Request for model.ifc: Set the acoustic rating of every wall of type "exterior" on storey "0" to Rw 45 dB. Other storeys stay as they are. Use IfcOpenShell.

First a look at what the model holds.

```python
import ifcopenshell
import ifcopenshell.util.element

model = ifcopenshell.open("model.ifc")
print(model.schema)
storey = next(s for s in model.by_type("IfcBuildingStorey") if s.Name == "0")
walls = [e for e in ifcopenshell.util.element.get_decomposition(storey) if e.is_a("IfcWall")]
seen = {}
for e in walls:
    element_type = ifcopenshell.util.element.get_type(e)
    key = (element_type.Name if element_type != e and element_type else None, ifcopenshell.util.element.get_pset(e, "Pset_WallCommon", "AcousticRating"))
    seen[key] = seen.get(key, 0) + 1
for (name, value), count in sorted(seen.items(), key=str):
    print(count, "x", name, "|", value)
```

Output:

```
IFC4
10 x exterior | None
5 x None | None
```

```python
import ifcopenshell
import ifcopenshell.api.pset
import ifcopenshell.util.element

model = ifcopenshell.open("model.ifc")

storey = next(s for s in model.by_type("IfcBuildingStorey") if s.Name == "0")
walls = [e for e in ifcopenshell.util.element.get_decomposition(storey) if e.is_a("IfcWall")]

count = 0
for e in walls:
    element_type = ifcopenshell.util.element.get_type(e)
    if element_type in (None, e) or element_type.Name != "exterior":
        continue
    # add_pset returns the element's existing set when there is one.
    pset = ifcopenshell.api.pset.add_pset(model, product=e, name="Pset_WallCommon")
    ifcopenshell.api.pset.edit_pset(model, pset=pset, properties={"AcousticRating": "Rw 45 dB"})
    count += 1

print(count, "walls updated")

model.write("model_updated.ifc")
```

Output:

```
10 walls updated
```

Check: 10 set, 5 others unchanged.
